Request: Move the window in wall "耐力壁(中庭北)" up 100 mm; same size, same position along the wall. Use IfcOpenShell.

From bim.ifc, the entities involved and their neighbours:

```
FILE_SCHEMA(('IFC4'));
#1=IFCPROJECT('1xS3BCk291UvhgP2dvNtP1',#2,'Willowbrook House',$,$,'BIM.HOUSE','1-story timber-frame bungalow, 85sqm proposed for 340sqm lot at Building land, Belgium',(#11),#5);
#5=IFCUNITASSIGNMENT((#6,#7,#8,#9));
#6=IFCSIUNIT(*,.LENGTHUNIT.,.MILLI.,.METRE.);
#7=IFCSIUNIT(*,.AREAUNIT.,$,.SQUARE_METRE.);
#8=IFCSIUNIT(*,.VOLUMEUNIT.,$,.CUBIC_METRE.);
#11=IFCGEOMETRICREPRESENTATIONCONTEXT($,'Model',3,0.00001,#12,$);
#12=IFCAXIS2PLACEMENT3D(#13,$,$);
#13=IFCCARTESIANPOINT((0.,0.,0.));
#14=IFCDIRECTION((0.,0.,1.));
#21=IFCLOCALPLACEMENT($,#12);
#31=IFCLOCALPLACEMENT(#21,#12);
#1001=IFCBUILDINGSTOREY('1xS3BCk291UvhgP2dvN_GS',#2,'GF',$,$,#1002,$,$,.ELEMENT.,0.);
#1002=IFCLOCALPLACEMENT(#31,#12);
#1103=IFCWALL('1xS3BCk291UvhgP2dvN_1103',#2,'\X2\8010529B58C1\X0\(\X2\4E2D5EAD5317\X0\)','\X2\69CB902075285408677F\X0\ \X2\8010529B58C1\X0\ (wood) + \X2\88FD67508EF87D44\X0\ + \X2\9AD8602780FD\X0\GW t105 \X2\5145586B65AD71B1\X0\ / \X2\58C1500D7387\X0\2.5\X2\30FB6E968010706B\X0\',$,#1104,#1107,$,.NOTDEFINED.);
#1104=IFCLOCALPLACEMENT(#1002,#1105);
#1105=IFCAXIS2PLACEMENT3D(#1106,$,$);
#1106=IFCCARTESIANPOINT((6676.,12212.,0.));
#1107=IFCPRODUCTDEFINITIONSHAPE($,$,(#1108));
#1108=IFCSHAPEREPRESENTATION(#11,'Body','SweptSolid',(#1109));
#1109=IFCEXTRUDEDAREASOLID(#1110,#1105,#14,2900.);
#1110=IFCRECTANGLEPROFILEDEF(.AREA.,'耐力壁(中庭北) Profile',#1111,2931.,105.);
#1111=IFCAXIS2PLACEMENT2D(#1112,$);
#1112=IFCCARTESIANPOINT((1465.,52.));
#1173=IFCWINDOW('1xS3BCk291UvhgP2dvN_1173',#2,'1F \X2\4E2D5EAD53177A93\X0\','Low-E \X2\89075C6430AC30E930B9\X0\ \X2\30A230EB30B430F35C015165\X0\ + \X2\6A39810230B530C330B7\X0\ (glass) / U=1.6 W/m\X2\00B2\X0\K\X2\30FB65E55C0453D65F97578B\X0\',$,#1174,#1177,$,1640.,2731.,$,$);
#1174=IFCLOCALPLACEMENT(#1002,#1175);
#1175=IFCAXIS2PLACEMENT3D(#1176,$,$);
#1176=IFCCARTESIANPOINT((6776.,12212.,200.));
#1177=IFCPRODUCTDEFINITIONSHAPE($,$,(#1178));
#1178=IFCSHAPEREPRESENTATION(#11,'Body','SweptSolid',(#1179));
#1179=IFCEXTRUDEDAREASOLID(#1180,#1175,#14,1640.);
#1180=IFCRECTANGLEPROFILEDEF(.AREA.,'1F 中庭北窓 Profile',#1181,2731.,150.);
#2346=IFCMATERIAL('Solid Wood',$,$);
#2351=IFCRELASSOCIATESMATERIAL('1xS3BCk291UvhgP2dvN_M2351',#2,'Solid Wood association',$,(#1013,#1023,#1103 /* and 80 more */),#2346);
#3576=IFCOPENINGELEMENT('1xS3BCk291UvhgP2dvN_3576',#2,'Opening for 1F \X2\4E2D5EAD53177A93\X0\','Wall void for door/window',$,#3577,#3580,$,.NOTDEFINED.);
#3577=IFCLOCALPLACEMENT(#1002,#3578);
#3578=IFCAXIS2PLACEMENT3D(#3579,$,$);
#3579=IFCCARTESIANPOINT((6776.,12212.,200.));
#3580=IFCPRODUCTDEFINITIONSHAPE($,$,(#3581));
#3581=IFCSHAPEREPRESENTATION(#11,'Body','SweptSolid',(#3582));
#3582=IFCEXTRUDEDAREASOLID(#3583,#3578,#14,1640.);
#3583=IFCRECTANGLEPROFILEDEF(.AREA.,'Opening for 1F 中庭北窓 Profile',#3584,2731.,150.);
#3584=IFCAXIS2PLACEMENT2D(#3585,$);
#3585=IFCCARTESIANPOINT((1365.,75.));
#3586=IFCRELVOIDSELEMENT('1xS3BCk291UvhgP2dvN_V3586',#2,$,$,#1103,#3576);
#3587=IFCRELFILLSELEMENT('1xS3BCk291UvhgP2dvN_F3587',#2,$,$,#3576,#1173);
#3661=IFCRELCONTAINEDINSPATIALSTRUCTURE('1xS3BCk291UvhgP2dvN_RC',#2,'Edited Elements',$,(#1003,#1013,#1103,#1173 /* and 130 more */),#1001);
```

```python
import numpy as np
import ifcopenshell
import ifcopenshell.api.geometry
import ifcopenshell.util.placement
import ifcopenshell.util.unit

model = ifcopenshell.open("bim.ifc")
unit_scale = ifcopenshell.util.unit.calculate_unit_scale(model)

window = model.by_id(1173)
opening = window.FillsVoids[0].RelatingOpeningElement
dz = 100.0

shift = np.array([0.0, 0.0, dz])
# The window is not placed relative to its opening, so move both.
for product in (opening, window):
    matrix = ifcopenshell.util.placement.get_local_placement(product.ObjectPlacement)
    matrix[:3, 3] += shift
    ifcopenshell.api.geometry.edit_object_placement(model, product=product, matrix=matrix, is_si=False)

print(f"moved by {dz * unit_scale:+.3f} m")

model.write("bim_rev.ifc")
```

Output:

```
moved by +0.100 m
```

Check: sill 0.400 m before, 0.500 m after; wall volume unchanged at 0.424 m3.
